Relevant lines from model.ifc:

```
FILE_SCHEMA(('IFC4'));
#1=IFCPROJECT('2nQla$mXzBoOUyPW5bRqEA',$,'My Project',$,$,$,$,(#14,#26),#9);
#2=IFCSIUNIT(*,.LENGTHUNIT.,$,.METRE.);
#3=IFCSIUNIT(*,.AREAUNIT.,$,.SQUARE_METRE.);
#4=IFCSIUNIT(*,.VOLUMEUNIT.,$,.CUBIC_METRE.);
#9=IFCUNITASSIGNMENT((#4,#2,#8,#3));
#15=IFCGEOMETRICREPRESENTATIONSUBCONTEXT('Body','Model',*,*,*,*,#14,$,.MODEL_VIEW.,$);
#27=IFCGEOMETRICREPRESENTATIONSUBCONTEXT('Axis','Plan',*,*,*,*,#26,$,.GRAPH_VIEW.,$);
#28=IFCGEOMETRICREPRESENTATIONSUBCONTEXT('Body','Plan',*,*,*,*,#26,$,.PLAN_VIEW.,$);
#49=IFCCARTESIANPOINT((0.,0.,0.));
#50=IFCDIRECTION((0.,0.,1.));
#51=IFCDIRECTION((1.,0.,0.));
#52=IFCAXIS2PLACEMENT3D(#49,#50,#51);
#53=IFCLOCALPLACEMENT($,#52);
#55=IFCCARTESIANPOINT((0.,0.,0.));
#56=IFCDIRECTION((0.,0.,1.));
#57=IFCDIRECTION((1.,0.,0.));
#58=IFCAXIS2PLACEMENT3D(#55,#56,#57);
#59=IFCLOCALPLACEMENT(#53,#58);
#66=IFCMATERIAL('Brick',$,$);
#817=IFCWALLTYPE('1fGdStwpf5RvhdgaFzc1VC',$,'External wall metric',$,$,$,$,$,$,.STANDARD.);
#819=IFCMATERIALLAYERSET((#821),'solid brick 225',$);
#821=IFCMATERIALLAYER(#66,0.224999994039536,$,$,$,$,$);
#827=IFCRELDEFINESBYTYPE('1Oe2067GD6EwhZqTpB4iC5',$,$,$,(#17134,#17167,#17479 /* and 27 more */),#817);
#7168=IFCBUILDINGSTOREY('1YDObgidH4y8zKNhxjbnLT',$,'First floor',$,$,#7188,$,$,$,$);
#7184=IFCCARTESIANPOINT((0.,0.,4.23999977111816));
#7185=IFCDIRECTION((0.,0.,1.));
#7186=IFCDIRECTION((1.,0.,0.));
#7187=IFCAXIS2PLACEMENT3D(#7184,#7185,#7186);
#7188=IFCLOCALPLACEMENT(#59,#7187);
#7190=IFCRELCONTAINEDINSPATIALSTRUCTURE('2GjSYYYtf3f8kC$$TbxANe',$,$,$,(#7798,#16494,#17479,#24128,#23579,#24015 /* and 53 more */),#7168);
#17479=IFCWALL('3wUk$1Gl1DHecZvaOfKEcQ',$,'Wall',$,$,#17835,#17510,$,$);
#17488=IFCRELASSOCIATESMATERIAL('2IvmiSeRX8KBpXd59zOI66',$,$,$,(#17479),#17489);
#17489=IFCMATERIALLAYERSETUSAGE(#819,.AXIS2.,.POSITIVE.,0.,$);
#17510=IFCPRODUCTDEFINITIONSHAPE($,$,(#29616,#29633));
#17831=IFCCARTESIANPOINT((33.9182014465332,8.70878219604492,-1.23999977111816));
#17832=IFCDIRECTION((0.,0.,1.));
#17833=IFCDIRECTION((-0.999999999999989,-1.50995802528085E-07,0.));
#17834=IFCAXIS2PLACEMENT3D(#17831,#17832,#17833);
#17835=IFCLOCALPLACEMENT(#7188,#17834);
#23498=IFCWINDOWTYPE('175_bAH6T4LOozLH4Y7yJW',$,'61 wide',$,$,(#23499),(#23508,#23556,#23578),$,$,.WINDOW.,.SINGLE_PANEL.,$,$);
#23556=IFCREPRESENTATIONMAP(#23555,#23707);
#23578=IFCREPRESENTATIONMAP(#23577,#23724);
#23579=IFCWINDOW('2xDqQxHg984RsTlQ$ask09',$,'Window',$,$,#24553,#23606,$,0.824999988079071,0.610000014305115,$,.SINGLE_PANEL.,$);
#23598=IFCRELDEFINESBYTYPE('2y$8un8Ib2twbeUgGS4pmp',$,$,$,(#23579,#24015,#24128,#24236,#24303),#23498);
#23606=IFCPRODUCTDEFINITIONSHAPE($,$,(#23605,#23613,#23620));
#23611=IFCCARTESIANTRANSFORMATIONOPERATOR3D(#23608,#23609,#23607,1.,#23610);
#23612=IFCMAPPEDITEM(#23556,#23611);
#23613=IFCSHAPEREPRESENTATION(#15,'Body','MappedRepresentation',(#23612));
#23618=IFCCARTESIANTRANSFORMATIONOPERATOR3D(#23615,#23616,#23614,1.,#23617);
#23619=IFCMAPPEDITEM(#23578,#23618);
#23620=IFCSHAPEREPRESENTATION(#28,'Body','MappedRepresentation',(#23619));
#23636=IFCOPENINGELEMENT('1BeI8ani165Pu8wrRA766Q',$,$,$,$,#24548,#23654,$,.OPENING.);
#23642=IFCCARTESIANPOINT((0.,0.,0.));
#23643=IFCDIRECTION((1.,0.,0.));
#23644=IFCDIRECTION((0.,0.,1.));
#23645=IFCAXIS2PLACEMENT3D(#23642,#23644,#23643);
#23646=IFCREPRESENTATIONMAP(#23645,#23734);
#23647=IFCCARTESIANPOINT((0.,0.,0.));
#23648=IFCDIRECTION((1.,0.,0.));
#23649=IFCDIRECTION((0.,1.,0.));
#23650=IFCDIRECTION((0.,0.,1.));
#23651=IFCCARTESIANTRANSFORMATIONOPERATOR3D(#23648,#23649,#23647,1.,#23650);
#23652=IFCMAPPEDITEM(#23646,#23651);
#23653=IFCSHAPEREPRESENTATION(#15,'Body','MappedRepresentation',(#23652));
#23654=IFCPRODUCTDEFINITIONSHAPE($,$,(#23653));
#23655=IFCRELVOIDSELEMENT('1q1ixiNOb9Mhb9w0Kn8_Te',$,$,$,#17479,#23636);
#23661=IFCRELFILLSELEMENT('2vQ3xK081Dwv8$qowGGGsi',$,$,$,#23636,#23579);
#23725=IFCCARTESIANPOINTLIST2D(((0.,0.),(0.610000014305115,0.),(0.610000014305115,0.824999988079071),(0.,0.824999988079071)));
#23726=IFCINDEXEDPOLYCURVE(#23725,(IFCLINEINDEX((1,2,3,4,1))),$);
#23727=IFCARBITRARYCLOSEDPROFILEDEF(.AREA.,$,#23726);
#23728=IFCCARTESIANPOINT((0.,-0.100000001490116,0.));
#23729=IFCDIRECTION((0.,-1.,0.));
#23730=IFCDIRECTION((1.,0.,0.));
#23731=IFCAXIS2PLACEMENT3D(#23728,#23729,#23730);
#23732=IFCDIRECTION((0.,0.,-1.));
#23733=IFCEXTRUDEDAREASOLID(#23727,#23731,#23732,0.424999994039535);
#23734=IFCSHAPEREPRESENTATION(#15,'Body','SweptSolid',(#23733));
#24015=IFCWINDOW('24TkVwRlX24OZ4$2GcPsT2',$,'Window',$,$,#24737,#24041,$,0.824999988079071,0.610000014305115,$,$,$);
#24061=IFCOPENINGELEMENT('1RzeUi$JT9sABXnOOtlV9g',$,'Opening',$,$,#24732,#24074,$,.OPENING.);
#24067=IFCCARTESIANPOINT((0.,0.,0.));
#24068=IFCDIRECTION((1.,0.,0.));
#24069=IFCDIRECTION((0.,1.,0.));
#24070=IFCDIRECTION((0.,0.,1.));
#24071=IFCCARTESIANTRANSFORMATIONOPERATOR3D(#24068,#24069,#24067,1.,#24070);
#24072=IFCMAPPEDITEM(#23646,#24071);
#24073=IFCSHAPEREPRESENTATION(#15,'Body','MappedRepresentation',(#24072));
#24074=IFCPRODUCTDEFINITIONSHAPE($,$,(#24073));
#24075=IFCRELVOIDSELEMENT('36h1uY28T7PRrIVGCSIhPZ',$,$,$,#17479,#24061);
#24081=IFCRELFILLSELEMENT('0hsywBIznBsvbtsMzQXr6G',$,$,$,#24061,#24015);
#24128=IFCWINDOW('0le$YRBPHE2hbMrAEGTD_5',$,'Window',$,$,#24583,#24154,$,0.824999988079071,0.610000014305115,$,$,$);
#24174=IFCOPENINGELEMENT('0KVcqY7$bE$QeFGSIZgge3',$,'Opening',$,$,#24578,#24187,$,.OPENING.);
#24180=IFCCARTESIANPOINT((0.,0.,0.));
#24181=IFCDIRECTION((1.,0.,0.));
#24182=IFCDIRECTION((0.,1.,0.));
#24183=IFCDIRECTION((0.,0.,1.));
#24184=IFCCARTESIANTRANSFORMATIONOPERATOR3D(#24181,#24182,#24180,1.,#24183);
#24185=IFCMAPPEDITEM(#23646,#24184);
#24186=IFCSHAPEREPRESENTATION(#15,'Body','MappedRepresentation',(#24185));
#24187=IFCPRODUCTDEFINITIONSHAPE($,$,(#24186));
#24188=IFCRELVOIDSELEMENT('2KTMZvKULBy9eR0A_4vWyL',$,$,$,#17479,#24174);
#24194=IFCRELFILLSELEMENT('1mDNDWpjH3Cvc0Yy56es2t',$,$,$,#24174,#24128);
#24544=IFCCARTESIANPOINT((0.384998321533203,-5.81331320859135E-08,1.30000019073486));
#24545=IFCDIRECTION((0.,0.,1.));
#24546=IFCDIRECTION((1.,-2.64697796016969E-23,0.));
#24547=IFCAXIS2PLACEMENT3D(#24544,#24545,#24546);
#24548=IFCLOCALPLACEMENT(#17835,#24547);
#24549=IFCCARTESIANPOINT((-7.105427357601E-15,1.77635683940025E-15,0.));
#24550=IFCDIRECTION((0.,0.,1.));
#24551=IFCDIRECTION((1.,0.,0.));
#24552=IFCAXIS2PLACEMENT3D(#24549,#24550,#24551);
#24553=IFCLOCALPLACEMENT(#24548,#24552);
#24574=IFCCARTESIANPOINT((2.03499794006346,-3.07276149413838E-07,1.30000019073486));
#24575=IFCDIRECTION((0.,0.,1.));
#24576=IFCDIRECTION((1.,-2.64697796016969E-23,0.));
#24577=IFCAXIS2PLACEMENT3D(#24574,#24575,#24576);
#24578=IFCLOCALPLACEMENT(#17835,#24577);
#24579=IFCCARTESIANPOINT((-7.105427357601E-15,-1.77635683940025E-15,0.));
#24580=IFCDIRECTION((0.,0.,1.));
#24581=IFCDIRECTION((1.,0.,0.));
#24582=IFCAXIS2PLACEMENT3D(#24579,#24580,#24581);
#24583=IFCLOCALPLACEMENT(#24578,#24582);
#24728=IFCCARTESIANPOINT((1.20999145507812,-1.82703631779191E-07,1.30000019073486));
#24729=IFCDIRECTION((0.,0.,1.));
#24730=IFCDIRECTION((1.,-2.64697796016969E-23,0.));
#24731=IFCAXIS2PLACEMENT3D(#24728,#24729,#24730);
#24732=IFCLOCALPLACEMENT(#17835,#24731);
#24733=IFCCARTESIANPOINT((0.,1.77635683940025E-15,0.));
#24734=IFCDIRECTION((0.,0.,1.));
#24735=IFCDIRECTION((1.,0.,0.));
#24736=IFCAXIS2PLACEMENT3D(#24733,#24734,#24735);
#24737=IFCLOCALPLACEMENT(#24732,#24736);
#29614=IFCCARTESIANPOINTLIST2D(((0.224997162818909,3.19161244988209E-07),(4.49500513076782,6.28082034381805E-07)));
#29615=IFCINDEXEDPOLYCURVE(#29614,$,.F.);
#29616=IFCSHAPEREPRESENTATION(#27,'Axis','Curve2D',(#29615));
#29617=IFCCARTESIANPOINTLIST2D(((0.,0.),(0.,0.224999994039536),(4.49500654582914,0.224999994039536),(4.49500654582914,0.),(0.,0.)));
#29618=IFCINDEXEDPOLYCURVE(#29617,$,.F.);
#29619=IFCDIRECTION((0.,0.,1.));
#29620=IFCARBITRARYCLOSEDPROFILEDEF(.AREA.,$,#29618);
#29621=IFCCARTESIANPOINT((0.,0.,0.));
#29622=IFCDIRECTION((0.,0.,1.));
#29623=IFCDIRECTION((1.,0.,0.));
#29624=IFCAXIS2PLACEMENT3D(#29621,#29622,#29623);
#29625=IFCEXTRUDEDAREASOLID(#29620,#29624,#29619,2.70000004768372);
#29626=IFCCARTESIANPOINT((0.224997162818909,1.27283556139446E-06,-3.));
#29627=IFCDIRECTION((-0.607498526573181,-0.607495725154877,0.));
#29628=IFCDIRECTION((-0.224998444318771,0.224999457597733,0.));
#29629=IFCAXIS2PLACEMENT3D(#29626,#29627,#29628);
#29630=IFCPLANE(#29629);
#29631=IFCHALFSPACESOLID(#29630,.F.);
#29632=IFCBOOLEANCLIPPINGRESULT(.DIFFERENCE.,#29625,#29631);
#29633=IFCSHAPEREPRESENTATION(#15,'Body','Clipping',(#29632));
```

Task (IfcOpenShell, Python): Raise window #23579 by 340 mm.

```python
import numpy as np
import ifcopenshell
import ifcopenshell.api.geometry
import ifcopenshell.util.placement
import ifcopenshell.util.unit

model = ifcopenshell.open("model.ifc")
unit_scale = ifcopenshell.util.unit.calculate_unit_scale(model)

window = model.by_id(23579)
opening = window.FillsVoids[0].RelatingOpeningElement
dz = 0.34 / unit_scale

shift = np.array([0.0, 0.0, dz])
# The window is placed relative to its opening, so it follows when the opening moves.
matrix = ifcopenshell.util.placement.get_local_placement(opening.ObjectPlacement)
matrix[:3, 3] += shift
ifcopenshell.api.geometry.edit_object_placement(
    model, product=opening, matrix=matrix, is_si=False, should_transform_children=True
)

print(f"moved by {dz * unit_scale:+.3f} m")

model.write("model_rev.ifc")
```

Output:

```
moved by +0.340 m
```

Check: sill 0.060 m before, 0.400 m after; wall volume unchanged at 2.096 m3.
